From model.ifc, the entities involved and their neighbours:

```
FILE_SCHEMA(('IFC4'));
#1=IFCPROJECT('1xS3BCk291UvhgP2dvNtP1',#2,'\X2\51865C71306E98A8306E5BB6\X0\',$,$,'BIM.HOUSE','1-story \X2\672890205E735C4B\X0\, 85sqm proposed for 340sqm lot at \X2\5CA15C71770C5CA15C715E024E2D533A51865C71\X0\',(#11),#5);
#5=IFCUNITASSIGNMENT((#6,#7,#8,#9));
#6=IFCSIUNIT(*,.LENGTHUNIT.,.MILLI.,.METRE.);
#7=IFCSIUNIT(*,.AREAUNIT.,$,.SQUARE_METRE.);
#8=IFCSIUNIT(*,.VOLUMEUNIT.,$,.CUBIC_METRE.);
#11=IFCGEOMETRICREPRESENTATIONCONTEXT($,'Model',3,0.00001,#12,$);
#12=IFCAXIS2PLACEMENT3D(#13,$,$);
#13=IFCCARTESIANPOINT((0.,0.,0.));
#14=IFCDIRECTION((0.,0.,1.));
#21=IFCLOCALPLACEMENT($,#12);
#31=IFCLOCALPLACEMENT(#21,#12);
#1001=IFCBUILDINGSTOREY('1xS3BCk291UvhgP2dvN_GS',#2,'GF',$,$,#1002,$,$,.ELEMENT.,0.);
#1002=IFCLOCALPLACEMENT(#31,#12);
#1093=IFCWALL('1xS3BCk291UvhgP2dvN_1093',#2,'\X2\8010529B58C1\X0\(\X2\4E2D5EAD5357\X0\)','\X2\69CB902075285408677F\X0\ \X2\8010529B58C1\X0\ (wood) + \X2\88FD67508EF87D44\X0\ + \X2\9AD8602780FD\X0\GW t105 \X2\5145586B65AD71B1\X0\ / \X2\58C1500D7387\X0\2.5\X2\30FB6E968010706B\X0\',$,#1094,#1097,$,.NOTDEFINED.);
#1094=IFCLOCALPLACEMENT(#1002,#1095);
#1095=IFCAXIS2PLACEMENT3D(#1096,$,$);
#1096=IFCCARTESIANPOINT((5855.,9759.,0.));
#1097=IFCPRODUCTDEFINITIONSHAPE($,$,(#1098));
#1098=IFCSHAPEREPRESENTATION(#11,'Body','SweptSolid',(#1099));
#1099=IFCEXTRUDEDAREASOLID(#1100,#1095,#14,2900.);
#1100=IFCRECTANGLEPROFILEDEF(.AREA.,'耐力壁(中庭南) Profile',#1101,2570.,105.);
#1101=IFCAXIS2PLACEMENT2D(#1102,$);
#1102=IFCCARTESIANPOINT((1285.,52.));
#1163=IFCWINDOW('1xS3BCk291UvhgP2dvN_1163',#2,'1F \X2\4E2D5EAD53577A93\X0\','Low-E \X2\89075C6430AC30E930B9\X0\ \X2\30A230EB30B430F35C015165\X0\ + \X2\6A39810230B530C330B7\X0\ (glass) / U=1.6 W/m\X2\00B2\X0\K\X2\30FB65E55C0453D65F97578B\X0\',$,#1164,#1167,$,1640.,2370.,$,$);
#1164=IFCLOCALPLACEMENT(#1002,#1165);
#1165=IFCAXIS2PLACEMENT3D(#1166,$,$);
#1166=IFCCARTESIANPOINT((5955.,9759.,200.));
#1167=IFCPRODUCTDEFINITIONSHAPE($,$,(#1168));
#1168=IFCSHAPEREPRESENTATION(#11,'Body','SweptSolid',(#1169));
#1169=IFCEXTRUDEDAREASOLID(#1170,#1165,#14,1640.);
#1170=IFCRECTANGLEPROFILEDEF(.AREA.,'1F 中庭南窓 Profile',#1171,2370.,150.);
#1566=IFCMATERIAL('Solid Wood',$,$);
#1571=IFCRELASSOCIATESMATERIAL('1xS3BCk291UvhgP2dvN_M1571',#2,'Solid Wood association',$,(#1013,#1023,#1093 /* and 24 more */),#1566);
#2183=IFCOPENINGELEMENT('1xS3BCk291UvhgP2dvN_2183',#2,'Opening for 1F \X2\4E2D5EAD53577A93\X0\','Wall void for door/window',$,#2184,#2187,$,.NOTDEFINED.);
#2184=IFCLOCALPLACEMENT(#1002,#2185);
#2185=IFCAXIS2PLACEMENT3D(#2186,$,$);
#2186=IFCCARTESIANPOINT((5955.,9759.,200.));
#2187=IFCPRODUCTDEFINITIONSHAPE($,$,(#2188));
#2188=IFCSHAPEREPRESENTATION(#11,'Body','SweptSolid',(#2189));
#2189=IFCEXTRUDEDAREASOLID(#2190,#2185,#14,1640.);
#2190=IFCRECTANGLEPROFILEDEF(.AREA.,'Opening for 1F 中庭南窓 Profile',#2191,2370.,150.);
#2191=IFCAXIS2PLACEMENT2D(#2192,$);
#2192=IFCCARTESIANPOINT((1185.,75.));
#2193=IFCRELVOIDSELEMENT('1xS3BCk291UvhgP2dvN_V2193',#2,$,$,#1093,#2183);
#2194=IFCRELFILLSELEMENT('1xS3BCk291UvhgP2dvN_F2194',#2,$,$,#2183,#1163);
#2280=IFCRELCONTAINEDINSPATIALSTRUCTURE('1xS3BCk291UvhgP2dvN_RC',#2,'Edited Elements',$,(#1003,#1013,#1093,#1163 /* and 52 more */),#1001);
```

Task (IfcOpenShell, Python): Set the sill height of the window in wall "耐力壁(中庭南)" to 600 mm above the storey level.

```python
import numpy as np
import ifcopenshell
import ifcopenshell.api.geometry
import ifcopenshell.geom
import ifcopenshell.util.element
import ifcopenshell.util.placement
import ifcopenshell.util.shape
import ifcopenshell.util.unit

model = ifcopenshell.open("model.ifc")
unit_scale = ifcopenshell.util.unit.calculate_unit_scale(model)

window = model.by_guid("1xS3BCk291UvhgP2dvN_1163")
opening = window.FillsVoids[0].RelatingOpeningElement
storey = ifcopenshell.util.element.get_container(window, ifc_class="IfcBuildingStorey")
level = ifcopenshell.util.placement.get_local_placement(storey.ObjectPlacement)[2, 3]

# The opening's origin need not be at the sill, so measure its lowest point.
shape = ifcopenshell.geom.create_shape(ifcopenshell.geom.settings(), opening)
bottom = ifcopenshell.util.shape.get_shape_bottom_elevation(shape, shape.geometry) / unit_scale
dz = level + 600.0 - bottom

shift = np.array([0.0, 0.0, dz])
# The window is not placed relative to its opening, so move both.
for product in (opening, window):
    matrix = ifcopenshell.util.placement.get_local_placement(product.ObjectPlacement)
    matrix[:3, 3] += shift
    ifcopenshell.api.geometry.edit_object_placement(model, product=product, matrix=matrix, is_si=False)

print(f"moved by {dz * unit_scale:+.3f} m")

model.write("model_rev.ifc")
```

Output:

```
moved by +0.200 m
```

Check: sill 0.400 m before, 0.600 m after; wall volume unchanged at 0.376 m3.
